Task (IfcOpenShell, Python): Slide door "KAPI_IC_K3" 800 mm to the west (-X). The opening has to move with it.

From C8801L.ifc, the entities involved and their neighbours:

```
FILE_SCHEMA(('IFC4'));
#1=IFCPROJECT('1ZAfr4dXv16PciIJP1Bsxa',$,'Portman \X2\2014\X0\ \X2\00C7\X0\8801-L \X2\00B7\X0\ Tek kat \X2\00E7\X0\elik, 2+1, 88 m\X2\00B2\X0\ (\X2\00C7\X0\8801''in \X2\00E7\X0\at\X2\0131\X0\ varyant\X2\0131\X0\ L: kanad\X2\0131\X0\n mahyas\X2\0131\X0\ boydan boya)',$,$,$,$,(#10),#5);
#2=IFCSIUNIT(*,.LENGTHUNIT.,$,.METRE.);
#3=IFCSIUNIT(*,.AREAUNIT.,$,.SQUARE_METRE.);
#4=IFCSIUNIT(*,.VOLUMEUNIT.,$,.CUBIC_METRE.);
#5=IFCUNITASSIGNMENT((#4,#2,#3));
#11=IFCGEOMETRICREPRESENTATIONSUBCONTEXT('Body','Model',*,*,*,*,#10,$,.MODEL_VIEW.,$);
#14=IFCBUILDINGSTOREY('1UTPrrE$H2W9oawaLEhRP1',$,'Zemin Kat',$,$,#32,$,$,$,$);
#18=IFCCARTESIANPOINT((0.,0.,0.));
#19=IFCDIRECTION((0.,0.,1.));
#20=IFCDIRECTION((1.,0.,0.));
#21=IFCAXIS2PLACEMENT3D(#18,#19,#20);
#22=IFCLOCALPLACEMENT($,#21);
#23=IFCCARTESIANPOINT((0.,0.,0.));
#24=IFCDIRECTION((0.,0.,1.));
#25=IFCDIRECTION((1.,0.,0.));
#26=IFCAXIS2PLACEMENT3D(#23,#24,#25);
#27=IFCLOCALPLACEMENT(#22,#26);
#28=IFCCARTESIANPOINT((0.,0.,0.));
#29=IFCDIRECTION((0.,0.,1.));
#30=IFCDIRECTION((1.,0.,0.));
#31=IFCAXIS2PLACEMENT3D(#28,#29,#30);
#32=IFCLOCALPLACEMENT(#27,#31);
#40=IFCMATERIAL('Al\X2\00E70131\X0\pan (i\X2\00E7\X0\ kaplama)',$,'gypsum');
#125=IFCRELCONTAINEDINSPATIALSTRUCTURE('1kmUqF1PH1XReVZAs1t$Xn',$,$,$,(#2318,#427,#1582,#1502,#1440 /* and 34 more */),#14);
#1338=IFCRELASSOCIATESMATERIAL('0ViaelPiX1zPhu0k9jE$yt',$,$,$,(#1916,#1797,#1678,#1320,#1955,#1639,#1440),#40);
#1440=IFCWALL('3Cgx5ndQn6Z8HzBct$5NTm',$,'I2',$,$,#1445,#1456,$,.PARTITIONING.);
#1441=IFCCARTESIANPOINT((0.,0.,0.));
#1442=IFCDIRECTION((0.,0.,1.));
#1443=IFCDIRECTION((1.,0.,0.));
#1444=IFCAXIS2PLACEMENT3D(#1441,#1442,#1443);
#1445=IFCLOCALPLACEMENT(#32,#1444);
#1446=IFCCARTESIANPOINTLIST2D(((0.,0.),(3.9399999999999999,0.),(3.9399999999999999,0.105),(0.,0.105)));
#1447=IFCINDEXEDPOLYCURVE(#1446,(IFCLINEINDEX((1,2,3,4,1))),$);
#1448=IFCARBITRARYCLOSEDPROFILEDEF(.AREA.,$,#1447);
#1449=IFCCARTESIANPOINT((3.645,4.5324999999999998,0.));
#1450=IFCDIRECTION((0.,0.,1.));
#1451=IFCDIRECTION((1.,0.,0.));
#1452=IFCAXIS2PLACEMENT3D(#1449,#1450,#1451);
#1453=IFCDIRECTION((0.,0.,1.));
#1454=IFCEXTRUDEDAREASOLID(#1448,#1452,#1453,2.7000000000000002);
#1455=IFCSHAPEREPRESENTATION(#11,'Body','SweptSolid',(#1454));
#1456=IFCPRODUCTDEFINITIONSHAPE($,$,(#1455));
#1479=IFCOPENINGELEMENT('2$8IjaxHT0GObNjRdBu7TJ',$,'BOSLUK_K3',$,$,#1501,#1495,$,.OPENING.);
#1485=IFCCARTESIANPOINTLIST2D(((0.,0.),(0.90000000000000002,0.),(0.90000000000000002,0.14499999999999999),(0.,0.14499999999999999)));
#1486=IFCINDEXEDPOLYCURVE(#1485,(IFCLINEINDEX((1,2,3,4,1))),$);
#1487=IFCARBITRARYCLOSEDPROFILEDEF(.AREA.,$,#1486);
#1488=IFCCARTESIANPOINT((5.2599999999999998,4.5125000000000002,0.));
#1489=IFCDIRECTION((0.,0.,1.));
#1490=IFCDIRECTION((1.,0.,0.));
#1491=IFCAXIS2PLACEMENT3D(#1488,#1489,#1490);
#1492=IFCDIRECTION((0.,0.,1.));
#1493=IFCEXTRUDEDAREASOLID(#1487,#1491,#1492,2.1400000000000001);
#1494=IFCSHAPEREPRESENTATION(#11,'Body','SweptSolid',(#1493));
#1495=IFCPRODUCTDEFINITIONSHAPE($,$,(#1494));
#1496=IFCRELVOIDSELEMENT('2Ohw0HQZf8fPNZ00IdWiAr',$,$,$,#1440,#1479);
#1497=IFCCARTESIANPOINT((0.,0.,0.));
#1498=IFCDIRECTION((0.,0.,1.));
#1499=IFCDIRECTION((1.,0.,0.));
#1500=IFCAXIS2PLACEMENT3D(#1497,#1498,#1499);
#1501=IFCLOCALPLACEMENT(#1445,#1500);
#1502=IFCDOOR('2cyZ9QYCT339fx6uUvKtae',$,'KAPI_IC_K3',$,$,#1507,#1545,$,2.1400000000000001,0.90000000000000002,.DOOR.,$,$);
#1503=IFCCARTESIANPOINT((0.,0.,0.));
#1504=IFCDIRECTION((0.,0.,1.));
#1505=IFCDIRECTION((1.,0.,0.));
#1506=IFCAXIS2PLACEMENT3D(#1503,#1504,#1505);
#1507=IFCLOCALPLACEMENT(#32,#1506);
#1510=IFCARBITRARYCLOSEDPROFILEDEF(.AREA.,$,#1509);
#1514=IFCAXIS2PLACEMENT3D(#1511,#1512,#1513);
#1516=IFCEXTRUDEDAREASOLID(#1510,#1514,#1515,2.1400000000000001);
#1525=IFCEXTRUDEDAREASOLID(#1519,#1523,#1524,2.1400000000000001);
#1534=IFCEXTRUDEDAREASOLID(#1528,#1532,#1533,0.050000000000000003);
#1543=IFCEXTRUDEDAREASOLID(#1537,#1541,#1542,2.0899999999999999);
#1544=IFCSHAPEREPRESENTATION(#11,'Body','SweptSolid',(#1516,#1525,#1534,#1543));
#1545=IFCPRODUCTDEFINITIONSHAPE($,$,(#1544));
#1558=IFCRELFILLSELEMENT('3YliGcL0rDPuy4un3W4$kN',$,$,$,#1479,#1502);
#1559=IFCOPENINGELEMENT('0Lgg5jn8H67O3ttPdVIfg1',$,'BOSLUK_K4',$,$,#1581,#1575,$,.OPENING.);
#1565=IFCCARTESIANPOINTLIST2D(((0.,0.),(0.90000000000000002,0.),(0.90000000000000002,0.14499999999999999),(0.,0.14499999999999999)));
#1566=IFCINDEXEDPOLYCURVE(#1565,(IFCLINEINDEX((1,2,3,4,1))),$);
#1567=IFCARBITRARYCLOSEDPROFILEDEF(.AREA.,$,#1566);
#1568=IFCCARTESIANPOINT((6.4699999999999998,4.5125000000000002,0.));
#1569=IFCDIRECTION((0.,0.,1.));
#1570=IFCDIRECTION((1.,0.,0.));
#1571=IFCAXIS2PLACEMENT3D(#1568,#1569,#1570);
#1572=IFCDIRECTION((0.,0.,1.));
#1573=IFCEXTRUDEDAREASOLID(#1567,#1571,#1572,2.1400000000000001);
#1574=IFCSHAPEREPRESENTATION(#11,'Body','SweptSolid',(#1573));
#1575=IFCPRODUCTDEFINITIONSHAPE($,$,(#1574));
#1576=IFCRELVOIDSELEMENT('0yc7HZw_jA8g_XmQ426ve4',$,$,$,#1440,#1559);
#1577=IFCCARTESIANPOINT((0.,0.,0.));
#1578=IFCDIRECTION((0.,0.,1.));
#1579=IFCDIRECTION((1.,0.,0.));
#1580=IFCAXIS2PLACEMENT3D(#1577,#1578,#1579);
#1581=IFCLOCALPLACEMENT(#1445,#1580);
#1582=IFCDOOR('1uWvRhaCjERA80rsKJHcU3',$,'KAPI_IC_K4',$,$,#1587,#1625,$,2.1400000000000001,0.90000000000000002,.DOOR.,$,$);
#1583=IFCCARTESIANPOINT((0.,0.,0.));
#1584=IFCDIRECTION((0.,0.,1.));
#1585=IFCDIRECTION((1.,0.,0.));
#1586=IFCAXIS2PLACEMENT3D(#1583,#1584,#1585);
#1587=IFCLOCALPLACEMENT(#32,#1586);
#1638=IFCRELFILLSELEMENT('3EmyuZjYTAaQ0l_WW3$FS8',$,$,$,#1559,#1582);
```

```python
import ifcopenshell
import ifcopenshell.api.geometry
import ifcopenshell.util.placement

model = ifcopenshell.open("C8801L.ifc")

door = model.by_guid("2cyZ9QYCT339fx6uUvKtae")
opening = door.FillsVoids[0].RelatingOpeningElement
wall = opening.VoidsElements[0].RelatingBuildingElement

wall_matrix = ifcopenshell.util.placement.get_local_placement(wall.ObjectPlacement)
shift = wall_matrix[:3, 0] * -0.8
before = ifcopenshell.util.placement.get_local_placement(door.ObjectPlacement)[:3, 3].copy()

# The door is not placed relative to its opening, so move both.
for product in (opening, door):
    matrix = ifcopenshell.util.placement.get_local_placement(product.ObjectPlacement)
    matrix[:3, 3] += shift
    ifcopenshell.api.geometry.edit_object_placement(model, product=product, matrix=matrix, is_si=False)

after = ifcopenshell.util.placement.get_local_placement(door.ObjectPlacement)[:3, 3]
print("door moved by", (after - before).round(3) + 0.0)

model.write("C8801L_updated.ifc")
```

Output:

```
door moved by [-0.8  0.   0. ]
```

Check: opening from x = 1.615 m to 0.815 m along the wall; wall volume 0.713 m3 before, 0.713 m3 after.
